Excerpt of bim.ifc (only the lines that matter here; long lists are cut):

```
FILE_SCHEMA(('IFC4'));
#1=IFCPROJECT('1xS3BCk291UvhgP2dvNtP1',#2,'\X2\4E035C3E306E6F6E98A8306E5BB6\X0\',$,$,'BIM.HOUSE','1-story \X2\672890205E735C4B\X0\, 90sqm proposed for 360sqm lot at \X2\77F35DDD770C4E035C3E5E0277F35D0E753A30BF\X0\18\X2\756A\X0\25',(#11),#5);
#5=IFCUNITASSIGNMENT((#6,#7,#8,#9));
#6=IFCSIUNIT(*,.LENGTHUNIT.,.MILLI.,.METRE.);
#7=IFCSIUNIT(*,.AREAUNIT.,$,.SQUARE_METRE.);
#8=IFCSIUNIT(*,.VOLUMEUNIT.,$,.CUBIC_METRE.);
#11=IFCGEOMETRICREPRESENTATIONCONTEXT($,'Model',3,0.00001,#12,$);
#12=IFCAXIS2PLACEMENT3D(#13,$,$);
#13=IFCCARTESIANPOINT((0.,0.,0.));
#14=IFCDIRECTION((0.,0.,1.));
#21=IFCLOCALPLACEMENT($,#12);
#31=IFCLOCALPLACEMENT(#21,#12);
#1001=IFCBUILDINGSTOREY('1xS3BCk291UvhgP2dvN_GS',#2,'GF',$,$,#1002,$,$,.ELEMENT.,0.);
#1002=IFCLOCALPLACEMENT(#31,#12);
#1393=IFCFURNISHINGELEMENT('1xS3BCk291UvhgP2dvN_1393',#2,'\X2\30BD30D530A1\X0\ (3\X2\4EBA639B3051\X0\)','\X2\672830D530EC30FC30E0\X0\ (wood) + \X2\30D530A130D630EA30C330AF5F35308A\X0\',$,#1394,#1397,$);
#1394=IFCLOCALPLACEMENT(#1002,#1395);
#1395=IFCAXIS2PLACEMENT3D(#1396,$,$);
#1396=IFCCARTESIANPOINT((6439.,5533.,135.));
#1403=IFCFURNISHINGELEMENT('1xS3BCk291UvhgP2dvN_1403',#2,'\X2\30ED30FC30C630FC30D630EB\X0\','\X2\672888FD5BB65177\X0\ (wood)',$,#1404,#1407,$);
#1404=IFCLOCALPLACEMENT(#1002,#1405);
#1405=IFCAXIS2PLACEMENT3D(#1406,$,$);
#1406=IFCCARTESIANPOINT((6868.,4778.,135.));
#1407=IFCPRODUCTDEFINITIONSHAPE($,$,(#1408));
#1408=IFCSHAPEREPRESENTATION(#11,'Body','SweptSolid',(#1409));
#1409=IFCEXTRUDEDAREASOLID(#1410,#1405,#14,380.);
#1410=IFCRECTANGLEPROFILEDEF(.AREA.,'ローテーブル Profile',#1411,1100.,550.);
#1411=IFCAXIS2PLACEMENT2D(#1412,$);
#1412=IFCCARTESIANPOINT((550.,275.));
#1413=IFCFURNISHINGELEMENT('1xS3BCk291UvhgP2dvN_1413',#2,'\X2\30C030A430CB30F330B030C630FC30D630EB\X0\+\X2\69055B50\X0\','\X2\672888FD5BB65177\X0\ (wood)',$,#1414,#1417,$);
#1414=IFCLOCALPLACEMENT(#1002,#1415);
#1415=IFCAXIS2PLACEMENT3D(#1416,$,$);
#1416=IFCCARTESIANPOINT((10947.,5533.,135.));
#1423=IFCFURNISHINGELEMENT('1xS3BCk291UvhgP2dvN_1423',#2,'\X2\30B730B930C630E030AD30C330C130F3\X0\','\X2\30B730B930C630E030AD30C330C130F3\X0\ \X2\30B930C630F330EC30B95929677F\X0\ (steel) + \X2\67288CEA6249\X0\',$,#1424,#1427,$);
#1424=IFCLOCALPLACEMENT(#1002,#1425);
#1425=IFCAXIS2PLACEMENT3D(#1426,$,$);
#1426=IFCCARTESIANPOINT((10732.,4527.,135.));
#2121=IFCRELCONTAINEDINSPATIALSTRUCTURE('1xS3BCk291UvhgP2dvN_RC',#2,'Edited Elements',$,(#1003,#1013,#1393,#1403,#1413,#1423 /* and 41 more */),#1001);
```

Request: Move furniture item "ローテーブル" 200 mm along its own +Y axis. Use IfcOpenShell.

```python
import ifcopenshell
import ifcopenshell.api.geometry
import ifcopenshell.util.placement
import ifcopenshell.util.unit

model = ifcopenshell.open("bim.ifc")
unit_scale = ifcopenshell.util.unit.calculate_unit_scale(model)

item = model.by_guid("1xS3BCk291UvhgP2dvN_1403")
matrix = ifcopenshell.util.placement.get_local_placement(item.ObjectPlacement)
matrix[:3, 3] += matrix[:3, 1] * 0.2 / unit_scale
ifcopenshell.api.geometry.edit_object_placement(model, product=item, matrix=matrix, is_si=False)

print(ifcopenshell.util.placement.get_local_placement(item.ObjectPlacement).round(3) + 0.0)

model.write("bim-out.ifc")
```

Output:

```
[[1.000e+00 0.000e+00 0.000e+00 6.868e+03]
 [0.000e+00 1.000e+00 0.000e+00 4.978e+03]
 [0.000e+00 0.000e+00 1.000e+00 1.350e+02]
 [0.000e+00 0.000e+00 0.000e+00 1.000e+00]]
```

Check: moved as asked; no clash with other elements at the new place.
